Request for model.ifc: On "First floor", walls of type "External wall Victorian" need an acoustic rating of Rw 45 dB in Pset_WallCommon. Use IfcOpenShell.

First a look at what the model holds.

```python
import ifcopenshell
import ifcopenshell.util.element

model = ifcopenshell.open("model.ifc")
print(model.schema)
storey = next(s for s in model.by_type("IfcBuildingStorey") if s.Name == "First floor")
walls = [e for e in ifcopenshell.util.element.get_decomposition(storey) if e.is_a("IfcWall")]
seen = {}
for e in walls:
    element_type = ifcopenshell.util.element.get_type(e)
    key = (element_type.Name if element_type != e and element_type else None, ifcopenshell.util.element.get_pset(e, "Pset_WallCommon", "AcousticRating"))
    seen[key] = seen.get(key, 0) + 1
for (name, value), count in sorted(seen.items(), key=str):
    print(count, "x", name, "|", value)
```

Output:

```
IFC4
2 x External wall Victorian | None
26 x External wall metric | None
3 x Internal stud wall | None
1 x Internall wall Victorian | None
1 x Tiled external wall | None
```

```python
import ifcopenshell
import ifcopenshell.api.pset
import ifcopenshell.util.element

model = ifcopenshell.open("model.ifc")

storey = next(s for s in model.by_type("IfcBuildingStorey") if s.Name == "First floor")
walls = [e for e in ifcopenshell.util.element.get_decomposition(storey) if e.is_a("IfcWall")]

count = 0
for e in walls:
    element_type = ifcopenshell.util.element.get_type(e)
    if element_type in (None, e) or element_type.Name != "External wall Victorian":
        continue
    # add_pset returns the element's existing set when there is one.
    pset = ifcopenshell.api.pset.add_pset(model, product=e, name="Pset_WallCommon")
    ifcopenshell.api.pset.edit_pset(model, pset=pset, properties={"AcousticRating": "Rw 45 dB"})
    count += 1

print(count, "walls updated")

model.write("model_edited.ifc")
```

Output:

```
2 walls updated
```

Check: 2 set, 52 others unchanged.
